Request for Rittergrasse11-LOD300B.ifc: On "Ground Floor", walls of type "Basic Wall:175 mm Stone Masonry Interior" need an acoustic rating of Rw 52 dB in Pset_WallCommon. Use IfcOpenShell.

First a look at what the model holds.

```python
import ifcopenshell
import ifcopenshell.util.element

model = ifcopenshell.open("Rittergrasse11-LOD300B.ifc")
print(model.schema)
storey = next(s for s in model.by_type("IfcBuildingStorey") if s.Name == "Ground Floor")
walls = [e for e in ifcopenshell.util.element.get_decomposition(storey) if e.is_a("IfcWall")]
seen = {}
for e in walls:
    element_type = ifcopenshell.util.element.get_type(e)
    key = (element_type.Name if element_type != e and element_type else None, ifcopenshell.util.element.get_pset(e, "Pset_WallCommon", "AcousticRating"))
    seen[key] = seen.get(key, 0) + 1
for (name, value), count in sorted(seen.items(), key=str):
    print(count, "x", name, "|", value)
```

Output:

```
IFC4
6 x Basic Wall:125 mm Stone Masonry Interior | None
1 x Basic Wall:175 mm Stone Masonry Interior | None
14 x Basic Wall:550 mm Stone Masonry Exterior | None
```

```python
import ifcopenshell
import ifcopenshell.api.pset
import ifcopenshell.util.element

model = ifcopenshell.open("Rittergrasse11-LOD300B.ifc")

storey = next(s for s in model.by_type("IfcBuildingStorey") if s.Name == "Ground Floor")
walls = [e for e in ifcopenshell.util.element.get_decomposition(storey) if e.is_a("IfcWall")]

count = 0
for e in walls:
    element_type = ifcopenshell.util.element.get_type(e)
    if element_type in (None, e) or element_type.Name != "Basic Wall:175 mm Stone Masonry Interior":
        continue
    # add_pset returns the element's existing set when there is one.
    pset = ifcopenshell.api.pset.add_pset(model, product=e, name="Pset_WallCommon")
    ifcopenshell.api.pset.edit_pset(model, pset=pset, properties={"AcousticRating": "Rw 52 dB"})
    count += 1

print(count, "walls updated")

model.write("Rittergrasse11-LOD300B_edited.ifc")
```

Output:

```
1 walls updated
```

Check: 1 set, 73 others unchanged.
